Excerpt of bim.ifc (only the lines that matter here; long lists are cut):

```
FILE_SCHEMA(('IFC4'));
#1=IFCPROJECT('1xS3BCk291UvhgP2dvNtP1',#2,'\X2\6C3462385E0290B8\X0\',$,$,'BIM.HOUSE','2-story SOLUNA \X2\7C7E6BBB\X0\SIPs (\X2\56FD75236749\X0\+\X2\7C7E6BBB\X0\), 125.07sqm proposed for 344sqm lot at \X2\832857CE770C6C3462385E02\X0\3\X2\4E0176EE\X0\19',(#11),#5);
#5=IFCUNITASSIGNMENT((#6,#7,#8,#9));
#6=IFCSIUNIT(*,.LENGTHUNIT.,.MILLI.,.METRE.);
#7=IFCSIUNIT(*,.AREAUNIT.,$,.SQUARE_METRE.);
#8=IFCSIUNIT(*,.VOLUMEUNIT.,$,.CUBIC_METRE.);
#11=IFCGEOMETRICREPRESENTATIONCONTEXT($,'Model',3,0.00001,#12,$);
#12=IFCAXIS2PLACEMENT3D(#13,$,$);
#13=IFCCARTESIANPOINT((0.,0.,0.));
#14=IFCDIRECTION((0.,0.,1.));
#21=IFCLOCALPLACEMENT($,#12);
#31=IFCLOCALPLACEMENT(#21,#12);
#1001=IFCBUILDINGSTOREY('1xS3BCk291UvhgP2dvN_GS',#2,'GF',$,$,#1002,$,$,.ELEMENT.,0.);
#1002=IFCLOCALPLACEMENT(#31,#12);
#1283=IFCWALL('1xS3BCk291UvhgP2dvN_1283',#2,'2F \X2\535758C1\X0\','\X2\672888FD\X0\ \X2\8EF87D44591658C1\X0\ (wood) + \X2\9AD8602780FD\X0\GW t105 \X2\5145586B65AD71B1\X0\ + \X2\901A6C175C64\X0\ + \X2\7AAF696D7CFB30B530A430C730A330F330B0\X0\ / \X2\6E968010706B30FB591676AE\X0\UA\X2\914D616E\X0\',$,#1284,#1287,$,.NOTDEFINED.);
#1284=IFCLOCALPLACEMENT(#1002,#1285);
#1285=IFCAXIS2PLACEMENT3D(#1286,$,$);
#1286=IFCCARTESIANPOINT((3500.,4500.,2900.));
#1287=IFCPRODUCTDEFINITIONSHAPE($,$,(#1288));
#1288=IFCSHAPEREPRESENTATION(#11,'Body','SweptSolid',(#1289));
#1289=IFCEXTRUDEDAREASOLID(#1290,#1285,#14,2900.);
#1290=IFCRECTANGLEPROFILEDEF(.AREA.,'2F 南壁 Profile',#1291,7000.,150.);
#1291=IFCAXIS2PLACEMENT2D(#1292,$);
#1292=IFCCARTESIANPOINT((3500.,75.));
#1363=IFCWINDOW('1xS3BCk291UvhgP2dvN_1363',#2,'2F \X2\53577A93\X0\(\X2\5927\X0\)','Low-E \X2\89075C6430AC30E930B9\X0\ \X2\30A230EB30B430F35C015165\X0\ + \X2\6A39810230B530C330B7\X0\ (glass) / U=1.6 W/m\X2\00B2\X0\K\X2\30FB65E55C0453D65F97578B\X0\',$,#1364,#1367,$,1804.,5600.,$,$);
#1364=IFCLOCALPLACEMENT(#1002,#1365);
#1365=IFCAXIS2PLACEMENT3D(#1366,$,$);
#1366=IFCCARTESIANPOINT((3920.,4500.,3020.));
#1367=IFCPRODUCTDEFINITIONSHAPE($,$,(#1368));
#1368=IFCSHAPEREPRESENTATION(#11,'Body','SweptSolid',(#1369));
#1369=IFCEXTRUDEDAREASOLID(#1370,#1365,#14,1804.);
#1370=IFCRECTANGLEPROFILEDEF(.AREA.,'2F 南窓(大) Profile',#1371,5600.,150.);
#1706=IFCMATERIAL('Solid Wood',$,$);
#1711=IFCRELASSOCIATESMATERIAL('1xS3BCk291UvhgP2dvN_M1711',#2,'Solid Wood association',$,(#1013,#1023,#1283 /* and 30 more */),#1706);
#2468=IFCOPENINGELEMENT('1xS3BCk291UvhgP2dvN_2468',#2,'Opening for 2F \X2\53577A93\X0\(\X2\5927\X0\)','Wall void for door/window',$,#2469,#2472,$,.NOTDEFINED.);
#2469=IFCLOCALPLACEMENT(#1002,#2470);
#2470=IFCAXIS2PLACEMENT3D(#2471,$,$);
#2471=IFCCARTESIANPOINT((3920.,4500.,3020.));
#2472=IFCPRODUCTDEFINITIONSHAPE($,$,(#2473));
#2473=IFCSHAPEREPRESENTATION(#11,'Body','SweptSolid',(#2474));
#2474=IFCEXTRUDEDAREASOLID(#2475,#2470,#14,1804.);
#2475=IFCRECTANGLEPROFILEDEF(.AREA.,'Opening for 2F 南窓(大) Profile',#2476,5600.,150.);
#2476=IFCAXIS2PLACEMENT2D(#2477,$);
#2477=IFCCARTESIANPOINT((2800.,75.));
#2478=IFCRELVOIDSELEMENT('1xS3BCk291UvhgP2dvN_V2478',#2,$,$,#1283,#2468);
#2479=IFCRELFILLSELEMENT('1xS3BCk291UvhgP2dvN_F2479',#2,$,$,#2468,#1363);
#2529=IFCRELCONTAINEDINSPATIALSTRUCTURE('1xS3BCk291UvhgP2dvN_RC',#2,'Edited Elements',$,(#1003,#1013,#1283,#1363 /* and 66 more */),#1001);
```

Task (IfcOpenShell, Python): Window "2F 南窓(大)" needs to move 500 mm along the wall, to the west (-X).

```python
import ifcopenshell
import ifcopenshell.api.geometry
import ifcopenshell.util.placement
import ifcopenshell.util.unit

model = ifcopenshell.open("bim.ifc")
unit_scale = ifcopenshell.util.unit.calculate_unit_scale(model)

window = model.by_guid("1xS3BCk291UvhgP2dvN_1363")
opening = window.FillsVoids[0].RelatingOpeningElement
wall = opening.VoidsElements[0].RelatingBuildingElement

wall_matrix = ifcopenshell.util.placement.get_local_placement(wall.ObjectPlacement)
shift = wall_matrix[:3, 0] * -0.5 / unit_scale
before = ifcopenshell.util.placement.get_local_placement(window.ObjectPlacement)[:3, 3].copy()

# The window is not placed relative to its opening, so move both.
for product in (opening, window):
    matrix = ifcopenshell.util.placement.get_local_placement(product.ObjectPlacement)
    matrix[:3, 3] += shift
    ifcopenshell.api.geometry.edit_object_placement(model, product=product, matrix=matrix, is_si=False)

after = ifcopenshell.util.placement.get_local_placement(window.ObjectPlacement)[:3, 3]
print("window moved by", (after - before).round(3) + 0.0)

model.write("bim_rev.ifc")
```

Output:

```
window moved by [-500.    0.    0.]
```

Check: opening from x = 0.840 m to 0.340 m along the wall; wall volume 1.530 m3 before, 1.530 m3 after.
